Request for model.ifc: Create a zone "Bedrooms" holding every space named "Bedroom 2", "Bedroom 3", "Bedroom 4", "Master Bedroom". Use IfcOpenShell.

First a look at what the model holds.

```python
import ifcopenshell

model = ifcopenshell.open("model.ifc")
print(model.schema)
seen = {}
for space in model.by_type("IfcSpace"):
    seen[space.LongName] = seen.get(space.LongName, 0) + 1
for name, count in sorted(seen.items(), key=str):
    print(count, "x", name)
print("zones:", [z.Name for z in model.by_type("IfcZone")][:20])
```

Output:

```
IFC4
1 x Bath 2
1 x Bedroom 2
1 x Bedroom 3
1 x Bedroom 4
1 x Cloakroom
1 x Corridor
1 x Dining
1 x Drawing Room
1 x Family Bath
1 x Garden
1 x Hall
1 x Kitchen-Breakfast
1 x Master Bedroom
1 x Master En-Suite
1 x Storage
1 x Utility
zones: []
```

```python
import ifcopenshell
import ifcopenshell.api.group
import ifcopenshell.api.root

model = ifcopenshell.open("model.ifc")

names = {"Bedroom 2", "Bedroom 3", "Bedroom 4", "Master Bedroom"}
spaces = [s for s in model.by_type("IfcSpace") if s.LongName in names]

zone = ifcopenshell.api.root.create_entity(model, ifc_class="IfcZone", name="Bedrooms")
ifcopenshell.api.group.assign_group(model, products=spaces, group=zone)
print(len(spaces), "spaces in", zone.Name)

model.write("model_updated.ifc")
```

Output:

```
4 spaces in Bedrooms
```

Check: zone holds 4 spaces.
